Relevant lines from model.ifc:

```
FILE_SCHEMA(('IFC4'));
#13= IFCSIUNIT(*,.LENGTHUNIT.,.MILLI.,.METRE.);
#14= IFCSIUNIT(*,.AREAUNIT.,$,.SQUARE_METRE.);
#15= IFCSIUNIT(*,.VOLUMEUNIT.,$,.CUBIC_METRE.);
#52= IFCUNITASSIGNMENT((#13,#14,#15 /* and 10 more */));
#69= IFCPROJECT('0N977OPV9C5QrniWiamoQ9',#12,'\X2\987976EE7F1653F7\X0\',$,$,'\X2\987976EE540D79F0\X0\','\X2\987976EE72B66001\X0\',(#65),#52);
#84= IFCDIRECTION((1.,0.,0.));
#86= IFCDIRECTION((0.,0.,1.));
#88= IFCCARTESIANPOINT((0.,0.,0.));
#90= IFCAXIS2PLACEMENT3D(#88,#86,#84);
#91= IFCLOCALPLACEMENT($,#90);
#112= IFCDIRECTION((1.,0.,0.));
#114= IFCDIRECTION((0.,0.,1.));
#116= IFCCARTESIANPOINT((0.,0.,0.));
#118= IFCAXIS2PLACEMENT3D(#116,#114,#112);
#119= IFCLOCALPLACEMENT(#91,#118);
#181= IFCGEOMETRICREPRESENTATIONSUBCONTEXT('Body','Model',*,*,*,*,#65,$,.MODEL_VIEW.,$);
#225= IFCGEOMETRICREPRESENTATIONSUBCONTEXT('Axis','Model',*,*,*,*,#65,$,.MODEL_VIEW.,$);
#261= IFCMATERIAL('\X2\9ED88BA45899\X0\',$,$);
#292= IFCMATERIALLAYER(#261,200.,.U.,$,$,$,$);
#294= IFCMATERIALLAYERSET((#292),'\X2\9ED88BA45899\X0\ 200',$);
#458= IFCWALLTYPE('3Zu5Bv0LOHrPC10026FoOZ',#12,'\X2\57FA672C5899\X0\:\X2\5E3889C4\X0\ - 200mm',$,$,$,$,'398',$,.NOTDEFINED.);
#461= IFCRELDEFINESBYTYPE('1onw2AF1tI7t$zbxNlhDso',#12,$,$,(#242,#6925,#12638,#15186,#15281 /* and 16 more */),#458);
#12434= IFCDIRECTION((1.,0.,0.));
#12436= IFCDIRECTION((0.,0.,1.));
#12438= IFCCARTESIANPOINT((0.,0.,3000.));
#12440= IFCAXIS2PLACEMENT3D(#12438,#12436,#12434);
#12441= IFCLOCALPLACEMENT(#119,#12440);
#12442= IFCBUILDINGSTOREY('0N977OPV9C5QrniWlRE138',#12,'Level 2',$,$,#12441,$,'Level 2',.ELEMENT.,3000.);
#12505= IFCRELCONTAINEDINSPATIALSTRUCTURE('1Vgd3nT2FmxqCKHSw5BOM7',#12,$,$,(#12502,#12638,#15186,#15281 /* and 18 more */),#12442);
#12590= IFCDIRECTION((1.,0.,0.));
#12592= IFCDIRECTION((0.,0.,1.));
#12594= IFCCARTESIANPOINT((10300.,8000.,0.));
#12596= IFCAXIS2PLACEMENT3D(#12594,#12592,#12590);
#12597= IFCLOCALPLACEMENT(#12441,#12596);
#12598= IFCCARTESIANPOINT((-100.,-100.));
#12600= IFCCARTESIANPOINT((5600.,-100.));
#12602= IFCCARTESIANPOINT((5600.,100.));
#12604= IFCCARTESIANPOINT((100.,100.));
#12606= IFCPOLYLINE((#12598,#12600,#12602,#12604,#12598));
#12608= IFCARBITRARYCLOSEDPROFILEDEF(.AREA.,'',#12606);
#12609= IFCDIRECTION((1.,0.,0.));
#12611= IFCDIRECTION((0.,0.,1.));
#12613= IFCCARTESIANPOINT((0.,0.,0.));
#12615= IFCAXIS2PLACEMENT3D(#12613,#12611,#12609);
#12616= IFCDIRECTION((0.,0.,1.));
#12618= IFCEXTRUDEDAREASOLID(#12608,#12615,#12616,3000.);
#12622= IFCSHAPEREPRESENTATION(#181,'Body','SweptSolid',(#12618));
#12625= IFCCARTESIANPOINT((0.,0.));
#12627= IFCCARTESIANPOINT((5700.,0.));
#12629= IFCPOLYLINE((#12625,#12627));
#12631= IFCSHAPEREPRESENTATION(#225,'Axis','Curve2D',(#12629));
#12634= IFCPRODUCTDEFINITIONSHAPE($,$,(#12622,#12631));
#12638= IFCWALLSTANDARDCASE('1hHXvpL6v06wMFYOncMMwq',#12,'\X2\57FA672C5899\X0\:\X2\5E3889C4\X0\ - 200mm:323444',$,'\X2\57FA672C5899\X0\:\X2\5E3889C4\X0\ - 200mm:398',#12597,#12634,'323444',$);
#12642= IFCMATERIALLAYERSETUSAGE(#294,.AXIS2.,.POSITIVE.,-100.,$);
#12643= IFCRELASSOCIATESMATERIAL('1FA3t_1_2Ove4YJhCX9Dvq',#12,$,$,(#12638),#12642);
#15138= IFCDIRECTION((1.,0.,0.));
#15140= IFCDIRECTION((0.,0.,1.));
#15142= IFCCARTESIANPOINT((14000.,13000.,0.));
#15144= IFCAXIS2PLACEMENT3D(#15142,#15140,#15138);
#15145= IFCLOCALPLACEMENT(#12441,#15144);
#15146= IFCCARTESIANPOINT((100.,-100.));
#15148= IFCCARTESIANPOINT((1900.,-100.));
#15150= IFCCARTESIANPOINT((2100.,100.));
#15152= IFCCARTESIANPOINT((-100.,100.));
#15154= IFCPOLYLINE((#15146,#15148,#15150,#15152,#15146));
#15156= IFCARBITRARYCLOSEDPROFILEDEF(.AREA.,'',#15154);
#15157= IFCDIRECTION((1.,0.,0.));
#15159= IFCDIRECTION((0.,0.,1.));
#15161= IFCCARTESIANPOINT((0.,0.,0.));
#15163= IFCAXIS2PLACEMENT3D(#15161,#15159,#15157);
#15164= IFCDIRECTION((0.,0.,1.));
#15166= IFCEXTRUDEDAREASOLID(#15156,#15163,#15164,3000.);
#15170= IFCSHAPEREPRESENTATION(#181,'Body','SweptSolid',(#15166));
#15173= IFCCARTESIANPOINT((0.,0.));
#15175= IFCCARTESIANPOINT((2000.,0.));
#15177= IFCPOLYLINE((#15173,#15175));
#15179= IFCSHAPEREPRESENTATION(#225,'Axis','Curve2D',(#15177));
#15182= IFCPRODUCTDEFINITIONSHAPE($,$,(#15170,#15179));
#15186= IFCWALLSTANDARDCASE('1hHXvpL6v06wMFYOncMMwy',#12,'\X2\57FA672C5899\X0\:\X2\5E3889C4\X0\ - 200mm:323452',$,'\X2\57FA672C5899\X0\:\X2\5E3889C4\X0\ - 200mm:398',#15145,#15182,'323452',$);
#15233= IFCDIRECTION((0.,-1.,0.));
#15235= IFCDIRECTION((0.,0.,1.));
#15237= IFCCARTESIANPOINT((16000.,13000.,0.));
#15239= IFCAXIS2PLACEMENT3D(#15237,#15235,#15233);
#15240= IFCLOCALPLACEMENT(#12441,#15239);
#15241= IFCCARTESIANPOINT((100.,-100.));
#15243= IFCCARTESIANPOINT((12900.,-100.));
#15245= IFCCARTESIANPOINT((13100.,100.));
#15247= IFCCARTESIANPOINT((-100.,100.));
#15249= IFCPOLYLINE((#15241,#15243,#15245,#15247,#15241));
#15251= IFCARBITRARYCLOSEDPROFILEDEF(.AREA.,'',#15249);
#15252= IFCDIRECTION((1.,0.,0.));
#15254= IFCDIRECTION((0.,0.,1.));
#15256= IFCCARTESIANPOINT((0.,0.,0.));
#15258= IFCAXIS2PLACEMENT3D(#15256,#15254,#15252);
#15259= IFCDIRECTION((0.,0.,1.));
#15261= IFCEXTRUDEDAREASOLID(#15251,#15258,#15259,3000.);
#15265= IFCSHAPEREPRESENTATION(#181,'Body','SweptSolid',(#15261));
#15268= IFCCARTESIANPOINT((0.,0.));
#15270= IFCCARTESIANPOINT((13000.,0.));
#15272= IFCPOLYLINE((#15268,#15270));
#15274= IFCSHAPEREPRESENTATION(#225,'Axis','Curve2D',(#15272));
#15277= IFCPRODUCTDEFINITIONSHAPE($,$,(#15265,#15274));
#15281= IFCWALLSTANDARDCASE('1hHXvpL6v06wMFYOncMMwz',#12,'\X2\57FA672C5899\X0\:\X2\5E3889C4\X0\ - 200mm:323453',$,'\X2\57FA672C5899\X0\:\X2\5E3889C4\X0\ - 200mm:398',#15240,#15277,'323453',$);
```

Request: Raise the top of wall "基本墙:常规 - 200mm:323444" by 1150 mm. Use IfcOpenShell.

```python
import ifcopenshell
import ifcopenshell.geom
import ifcopenshell.util.representation
import ifcopenshell.util.shape

model = ifcopenshell.open("model.ifc")
settings = ifcopenshell.geom.settings()


def volume(element):
    """Net volume in cubic metres, openings subtracted."""
    shape = ifcopenshell.geom.create_shape(settings, element)
    return ifcopenshell.util.shape.get_volume(shape.geometry)


wall = model.by_id(12638)
before = volume(wall)

body = ifcopenshell.util.representation.get_representation(wall, "Model", "Body")
solid = body.Items[0]
old_height = solid.Depth
solid.Depth += 1150.0
after = volume(wall)

print(f"height {old_height:g} -> {solid.Depth:g}, volume {before:.3f} -> {after:.3f} m3")

model.write("model_edited.ifc")
```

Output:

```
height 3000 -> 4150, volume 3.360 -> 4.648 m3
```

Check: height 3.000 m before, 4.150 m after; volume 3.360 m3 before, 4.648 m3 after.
